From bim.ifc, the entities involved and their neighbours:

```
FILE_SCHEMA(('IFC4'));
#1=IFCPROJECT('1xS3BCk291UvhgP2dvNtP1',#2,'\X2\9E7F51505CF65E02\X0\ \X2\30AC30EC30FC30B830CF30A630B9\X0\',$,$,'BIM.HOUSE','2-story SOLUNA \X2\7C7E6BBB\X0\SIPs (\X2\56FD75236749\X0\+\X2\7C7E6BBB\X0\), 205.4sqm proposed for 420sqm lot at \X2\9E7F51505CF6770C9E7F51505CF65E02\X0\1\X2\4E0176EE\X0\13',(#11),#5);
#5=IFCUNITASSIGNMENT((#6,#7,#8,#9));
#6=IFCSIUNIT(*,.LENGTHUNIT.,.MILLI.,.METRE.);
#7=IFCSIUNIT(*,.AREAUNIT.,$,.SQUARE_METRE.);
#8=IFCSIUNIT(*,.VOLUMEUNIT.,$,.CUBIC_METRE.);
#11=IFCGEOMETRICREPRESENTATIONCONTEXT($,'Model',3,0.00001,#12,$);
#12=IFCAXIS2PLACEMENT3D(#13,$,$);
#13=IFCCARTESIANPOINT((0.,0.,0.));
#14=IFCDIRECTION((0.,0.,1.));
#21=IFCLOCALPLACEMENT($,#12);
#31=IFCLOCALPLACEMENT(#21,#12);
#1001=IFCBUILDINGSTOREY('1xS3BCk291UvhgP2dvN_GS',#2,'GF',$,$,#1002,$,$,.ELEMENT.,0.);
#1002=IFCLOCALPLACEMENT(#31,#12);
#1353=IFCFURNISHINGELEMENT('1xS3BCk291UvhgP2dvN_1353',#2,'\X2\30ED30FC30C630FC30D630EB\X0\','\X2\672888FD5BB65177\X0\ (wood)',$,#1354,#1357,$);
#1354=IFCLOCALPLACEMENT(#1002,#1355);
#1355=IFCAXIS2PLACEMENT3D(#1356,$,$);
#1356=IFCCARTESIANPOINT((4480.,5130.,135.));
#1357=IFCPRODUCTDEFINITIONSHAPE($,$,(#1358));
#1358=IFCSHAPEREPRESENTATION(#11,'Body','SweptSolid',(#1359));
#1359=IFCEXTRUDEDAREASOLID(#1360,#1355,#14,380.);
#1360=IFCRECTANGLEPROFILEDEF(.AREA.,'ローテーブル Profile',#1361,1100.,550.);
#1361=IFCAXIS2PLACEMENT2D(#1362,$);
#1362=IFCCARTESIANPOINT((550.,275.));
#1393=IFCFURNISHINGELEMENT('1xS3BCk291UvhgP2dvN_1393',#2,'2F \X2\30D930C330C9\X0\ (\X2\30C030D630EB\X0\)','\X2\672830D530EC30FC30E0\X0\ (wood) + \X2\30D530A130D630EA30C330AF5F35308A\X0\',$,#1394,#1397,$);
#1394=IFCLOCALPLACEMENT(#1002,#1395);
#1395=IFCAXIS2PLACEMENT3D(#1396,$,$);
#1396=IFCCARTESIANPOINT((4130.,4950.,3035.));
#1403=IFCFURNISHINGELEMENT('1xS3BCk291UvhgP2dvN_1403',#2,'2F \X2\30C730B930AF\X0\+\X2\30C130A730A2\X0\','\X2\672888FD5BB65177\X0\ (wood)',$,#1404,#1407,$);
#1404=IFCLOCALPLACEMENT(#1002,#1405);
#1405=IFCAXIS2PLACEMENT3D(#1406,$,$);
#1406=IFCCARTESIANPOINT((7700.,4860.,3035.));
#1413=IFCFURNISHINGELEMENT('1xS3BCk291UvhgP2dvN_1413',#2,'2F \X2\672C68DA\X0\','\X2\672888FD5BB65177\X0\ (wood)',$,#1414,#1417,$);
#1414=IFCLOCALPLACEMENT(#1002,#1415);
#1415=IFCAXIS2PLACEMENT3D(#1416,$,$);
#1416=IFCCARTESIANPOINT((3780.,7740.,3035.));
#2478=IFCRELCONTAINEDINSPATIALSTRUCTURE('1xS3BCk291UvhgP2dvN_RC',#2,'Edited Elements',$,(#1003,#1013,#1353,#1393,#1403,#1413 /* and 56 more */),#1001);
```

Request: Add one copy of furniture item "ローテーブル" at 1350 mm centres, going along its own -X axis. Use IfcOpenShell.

```python
import ifcopenshell
import ifcopenshell.api.geometry
import ifcopenshell.api.root
import ifcopenshell.util.element
import ifcopenshell.util.placement

model = ifcopenshell.open("bim.ifc")


def reuse_history(source, copy):
    """copy_class also copies each property set's owner history, people and application; keep the originals."""
    for rel in copy.IsDefinedBy:
        if rel.is_a("IfcRelDefinesByProperties") and (history := rel.RelatingPropertyDefinition.OwnerHistory):
            rel.RelatingPropertyDefinition.OwnerHistory = source.OwnerHistory
            ifcopenshell.util.element.remove_deep2(model, history)


source = model.by_id(1353)
base = ifcopenshell.util.placement.get_local_placement(source.ObjectPlacement)
step = -base[:3, 0] * 1350.0

for i in range(1, 2):
    copy = ifcopenshell.api.root.copy_class(model, product=source)
    copy.Representation = ifcopenshell.util.element.copy_deep(
        model, source.Representation, exclude=["IfcGeometricRepresentationContext", "IfcRepresentationMap"]
    )
    reuse_history(source, copy)
    matrix = base.copy()
    matrix[:3, 3] += i * step
    print("added at", matrix[:3, 3].round(3) + 0.0)
    ifcopenshell.api.geometry.edit_object_placement(model, product=copy, matrix=matrix, is_si=False)

model.write("bim_rev.ifc")
```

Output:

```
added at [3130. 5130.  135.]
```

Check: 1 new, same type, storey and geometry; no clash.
